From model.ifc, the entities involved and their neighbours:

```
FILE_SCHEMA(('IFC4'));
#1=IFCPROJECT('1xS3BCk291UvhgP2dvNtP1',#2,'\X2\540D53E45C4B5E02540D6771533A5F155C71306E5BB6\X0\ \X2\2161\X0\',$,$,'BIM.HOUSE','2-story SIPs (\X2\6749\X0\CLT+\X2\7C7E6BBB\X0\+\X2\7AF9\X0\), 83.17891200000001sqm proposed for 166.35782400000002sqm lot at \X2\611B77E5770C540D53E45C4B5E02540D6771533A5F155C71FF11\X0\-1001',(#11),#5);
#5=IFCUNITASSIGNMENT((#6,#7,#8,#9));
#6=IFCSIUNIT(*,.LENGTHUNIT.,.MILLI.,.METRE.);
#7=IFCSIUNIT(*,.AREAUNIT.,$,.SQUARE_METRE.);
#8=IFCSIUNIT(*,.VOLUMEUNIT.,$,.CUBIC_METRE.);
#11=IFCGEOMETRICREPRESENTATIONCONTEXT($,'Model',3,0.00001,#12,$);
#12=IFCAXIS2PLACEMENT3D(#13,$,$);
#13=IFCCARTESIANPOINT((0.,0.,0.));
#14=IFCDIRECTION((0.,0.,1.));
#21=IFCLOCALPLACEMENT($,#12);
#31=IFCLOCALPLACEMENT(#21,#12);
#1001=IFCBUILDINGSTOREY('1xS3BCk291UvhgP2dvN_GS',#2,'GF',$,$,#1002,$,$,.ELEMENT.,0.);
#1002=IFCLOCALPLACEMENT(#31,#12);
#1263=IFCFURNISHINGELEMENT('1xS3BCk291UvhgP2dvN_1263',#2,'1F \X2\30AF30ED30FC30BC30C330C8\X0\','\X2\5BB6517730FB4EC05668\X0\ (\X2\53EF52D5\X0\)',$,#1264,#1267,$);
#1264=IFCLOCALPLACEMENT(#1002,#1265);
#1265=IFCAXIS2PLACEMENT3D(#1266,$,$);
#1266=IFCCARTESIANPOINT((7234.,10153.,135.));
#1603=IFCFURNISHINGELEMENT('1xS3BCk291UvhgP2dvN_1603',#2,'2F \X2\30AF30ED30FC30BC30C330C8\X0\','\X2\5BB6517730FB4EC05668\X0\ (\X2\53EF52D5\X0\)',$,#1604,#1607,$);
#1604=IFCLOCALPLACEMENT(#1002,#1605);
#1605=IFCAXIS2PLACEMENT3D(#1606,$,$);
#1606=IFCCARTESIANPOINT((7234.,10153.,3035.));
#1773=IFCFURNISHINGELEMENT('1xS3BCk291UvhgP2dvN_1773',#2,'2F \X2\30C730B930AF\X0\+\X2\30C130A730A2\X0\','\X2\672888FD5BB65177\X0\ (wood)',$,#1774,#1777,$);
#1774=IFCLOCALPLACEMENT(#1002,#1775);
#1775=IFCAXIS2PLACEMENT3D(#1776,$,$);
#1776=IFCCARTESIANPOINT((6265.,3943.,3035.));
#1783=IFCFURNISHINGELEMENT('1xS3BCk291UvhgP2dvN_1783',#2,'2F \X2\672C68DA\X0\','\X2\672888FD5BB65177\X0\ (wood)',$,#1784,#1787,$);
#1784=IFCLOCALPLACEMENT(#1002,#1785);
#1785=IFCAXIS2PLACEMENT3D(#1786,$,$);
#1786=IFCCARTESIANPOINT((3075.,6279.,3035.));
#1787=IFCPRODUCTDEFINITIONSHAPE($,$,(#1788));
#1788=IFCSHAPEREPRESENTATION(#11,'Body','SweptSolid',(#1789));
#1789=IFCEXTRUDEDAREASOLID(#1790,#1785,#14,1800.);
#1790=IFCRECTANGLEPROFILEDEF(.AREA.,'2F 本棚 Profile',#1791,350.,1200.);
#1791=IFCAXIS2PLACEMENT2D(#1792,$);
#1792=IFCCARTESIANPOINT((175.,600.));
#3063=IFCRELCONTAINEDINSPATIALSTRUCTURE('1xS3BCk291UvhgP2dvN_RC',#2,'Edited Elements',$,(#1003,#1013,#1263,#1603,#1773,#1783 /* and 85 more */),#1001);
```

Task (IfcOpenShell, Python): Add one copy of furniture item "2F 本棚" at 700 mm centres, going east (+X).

```python
import numpy as np
import ifcopenshell
import ifcopenshell.api.geometry
import ifcopenshell.api.root
import ifcopenshell.util.element
import ifcopenshell.util.placement

model = ifcopenshell.open("model.ifc")


def reuse_history(source, copy):
    """copy_class also copies each property set's owner history, people and application; keep the originals."""
    for rel in copy.IsDefinedBy:
        if rel.is_a("IfcRelDefinesByProperties") and (history := rel.RelatingPropertyDefinition.OwnerHistory):
            rel.RelatingPropertyDefinition.OwnerHistory = source.OwnerHistory
            ifcopenshell.util.element.remove_deep2(model, history)


source = model.by_guid("1xS3BCk291UvhgP2dvN_1783")
base = ifcopenshell.util.placement.get_local_placement(source.ObjectPlacement)
step = np.array([1.0, 0.0, 0.0]) * 700.0

for i in range(1, 2):
    copy = ifcopenshell.api.root.copy_class(model, product=source)
    copy.Representation = ifcopenshell.util.element.copy_deep(
        model, source.Representation, exclude=["IfcGeometricRepresentationContext", "IfcRepresentationMap"]
    )
    reuse_history(source, copy)
    matrix = base.copy()
    matrix[:3, 3] += i * step
    print("added at", matrix[:3, 3].round(3) + 0.0)
    ifcopenshell.api.geometry.edit_object_placement(model, product=copy, matrix=matrix, is_si=False)

model.write("model-out.ifc")
```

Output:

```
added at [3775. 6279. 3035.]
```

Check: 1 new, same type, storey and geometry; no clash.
